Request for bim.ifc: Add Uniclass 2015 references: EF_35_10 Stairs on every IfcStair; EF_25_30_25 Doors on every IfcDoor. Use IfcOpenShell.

First a look at what the model holds.

```python
import ifcopenshell

model = ifcopenshell.open("bim.ifc")
print(model.schema)
print("classifications:", [c.Name for c in model.by_type("IfcClassification")])
for ifc_class in ("IfcDoor", "IfcRoof", "IfcStair", "IfcWall", "IfcWindow"):
    print(ifc_class, len(model.by_type(ifc_class)))
```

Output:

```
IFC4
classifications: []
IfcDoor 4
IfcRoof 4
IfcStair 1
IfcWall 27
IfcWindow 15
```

```python
import ifcopenshell
import ifcopenshell.api.classification

model = ifcopenshell.open("bim.ifc")

system = ifcopenshell.api.classification.add_classification(model, classification="Uniclass 2015")

codes = {
    "IfcStair": ("EF_35_10", "Stairs"),
    "IfcDoor": ("EF_25_30_25", "Doors"),
}
for ifc_class, (code, name) in codes.items():
    products = model.by_type(ifc_class)
    ifcopenshell.api.classification.add_reference(
        model, products=products, classification=system, identification=code, name=name
    )
    print(code, len(products))

model.write("bim_edited.ifc")
```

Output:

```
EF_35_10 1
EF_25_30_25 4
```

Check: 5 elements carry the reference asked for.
